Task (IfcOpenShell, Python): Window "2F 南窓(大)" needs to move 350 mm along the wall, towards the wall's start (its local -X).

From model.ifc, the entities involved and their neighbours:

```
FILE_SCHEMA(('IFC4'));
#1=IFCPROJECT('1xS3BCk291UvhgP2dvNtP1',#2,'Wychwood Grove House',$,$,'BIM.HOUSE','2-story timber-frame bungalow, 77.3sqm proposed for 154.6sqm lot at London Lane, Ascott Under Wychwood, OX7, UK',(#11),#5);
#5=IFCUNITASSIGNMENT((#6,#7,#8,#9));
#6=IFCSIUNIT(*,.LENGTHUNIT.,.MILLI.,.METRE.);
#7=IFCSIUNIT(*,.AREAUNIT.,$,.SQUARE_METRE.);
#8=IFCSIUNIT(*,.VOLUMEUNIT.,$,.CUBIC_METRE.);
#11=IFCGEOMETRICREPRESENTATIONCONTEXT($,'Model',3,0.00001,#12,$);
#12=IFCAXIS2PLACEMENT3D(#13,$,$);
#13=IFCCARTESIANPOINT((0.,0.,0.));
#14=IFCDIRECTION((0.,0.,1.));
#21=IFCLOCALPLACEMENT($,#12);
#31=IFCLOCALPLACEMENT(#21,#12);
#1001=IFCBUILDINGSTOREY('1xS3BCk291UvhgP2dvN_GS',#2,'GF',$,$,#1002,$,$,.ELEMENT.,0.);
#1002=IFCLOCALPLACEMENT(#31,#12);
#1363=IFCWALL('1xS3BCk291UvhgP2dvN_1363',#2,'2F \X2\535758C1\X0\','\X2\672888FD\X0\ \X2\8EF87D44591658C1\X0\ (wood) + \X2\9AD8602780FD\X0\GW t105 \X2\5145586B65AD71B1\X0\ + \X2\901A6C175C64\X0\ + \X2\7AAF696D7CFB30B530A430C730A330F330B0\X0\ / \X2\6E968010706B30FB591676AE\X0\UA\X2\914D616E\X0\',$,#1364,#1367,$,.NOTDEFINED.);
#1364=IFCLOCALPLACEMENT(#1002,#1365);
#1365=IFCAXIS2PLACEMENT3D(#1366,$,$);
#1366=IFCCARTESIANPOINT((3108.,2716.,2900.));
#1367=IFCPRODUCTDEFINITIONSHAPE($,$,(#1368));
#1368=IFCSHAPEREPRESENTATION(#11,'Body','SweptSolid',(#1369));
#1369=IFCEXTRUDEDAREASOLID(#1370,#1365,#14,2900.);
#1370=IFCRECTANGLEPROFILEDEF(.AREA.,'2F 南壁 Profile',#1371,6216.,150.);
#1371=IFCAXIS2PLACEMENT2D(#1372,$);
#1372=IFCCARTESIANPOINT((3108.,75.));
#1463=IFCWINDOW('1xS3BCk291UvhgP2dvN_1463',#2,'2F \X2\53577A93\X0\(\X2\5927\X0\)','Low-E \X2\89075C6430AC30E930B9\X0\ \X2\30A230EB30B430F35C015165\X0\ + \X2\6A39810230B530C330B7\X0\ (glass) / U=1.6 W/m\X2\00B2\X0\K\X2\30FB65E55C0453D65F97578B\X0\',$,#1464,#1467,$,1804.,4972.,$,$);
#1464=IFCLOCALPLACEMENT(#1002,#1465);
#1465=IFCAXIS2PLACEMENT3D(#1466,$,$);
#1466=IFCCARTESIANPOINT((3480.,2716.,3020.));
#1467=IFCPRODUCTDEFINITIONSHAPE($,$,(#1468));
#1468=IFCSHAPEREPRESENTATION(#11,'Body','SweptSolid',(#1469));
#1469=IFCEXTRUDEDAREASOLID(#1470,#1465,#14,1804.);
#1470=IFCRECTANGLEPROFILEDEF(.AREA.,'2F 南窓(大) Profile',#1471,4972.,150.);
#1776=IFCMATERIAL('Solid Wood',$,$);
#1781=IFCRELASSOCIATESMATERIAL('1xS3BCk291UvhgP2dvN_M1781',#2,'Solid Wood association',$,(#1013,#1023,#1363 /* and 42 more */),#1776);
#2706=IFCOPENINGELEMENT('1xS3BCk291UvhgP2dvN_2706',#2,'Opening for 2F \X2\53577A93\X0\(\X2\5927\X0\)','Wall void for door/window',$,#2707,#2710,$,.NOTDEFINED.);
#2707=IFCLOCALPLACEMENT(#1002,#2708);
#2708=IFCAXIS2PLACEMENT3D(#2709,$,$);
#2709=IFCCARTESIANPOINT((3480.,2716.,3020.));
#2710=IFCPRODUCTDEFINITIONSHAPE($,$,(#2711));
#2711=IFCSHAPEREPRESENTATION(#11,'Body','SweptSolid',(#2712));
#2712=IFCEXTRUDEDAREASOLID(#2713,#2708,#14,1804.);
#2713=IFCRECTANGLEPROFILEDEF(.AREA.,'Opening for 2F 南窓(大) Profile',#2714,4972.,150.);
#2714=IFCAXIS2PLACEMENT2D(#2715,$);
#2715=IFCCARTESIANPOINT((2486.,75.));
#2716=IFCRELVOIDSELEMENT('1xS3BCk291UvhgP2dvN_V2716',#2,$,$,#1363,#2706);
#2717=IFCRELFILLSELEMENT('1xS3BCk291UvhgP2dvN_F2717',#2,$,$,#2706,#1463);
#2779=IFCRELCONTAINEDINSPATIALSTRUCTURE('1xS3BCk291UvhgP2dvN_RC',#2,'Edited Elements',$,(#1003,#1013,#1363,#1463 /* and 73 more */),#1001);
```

```python
import ifcopenshell
import ifcopenshell.api.geometry
import ifcopenshell.util.placement
import ifcopenshell.util.unit

model = ifcopenshell.open("model.ifc")
unit_scale = ifcopenshell.util.unit.calculate_unit_scale(model)

window = model.by_guid("1xS3BCk291UvhgP2dvN_1463")
opening = window.FillsVoids[0].RelatingOpeningElement
wall = opening.VoidsElements[0].RelatingBuildingElement

wall_matrix = ifcopenshell.util.placement.get_local_placement(wall.ObjectPlacement)
shift = wall_matrix[:3, 0] * -0.35 / unit_scale
before = ifcopenshell.util.placement.get_local_placement(window.ObjectPlacement)[:3, 3].copy()

# The window is not placed relative to its opening, so move both.
for product in (opening, window):
    matrix = ifcopenshell.util.placement.get_local_placement(product.ObjectPlacement)
    matrix[:3, 3] += shift
    ifcopenshell.api.geometry.edit_object_placement(model, product=product, matrix=matrix, is_si=False)

after = ifcopenshell.util.placement.get_local_placement(window.ObjectPlacement)[:3, 3]
print("window moved by", (after - before).round(3) + 0.0)

model.write("model_v2.ifc")
```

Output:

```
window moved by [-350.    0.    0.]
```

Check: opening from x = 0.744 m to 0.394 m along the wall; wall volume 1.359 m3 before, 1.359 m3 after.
